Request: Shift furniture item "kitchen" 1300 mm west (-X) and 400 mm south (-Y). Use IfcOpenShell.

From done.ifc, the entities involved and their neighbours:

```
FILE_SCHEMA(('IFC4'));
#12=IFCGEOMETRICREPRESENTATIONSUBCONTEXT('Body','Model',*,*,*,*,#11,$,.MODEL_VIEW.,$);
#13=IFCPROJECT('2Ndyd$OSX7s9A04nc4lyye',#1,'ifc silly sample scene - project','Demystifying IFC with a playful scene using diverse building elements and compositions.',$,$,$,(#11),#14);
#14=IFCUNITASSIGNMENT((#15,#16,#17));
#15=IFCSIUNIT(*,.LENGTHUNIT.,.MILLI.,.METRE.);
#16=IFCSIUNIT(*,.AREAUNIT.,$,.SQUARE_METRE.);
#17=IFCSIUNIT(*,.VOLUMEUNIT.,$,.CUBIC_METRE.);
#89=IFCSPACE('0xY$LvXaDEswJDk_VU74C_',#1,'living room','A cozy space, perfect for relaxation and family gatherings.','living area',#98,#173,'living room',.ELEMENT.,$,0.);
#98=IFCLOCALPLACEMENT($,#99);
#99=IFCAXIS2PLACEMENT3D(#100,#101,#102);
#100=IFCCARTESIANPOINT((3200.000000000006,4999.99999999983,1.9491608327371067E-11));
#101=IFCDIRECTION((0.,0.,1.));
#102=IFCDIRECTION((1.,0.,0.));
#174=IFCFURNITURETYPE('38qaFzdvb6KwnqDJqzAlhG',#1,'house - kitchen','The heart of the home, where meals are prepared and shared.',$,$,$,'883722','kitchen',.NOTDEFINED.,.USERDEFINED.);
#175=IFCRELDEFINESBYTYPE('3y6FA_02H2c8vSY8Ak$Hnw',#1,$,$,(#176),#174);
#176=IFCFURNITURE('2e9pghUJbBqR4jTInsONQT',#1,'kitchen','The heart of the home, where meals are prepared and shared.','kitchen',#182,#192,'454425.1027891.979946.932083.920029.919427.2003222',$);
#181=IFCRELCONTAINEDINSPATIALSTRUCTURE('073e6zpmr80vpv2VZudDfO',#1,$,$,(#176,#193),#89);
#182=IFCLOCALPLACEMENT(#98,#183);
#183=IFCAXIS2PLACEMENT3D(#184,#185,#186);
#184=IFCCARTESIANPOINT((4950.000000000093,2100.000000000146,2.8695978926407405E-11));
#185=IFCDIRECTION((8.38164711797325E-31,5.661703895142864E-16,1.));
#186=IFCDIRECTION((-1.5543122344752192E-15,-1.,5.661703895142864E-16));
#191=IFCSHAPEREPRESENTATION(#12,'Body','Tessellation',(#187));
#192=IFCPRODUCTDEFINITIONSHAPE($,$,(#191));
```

```python
import ifcopenshell
import ifcopenshell.api.geometry
import ifcopenshell.util.placement
import ifcopenshell.util.unit

model = ifcopenshell.open("done.ifc")
unit_scale = ifcopenshell.util.unit.calculate_unit_scale(model)

item = model.by_guid("2e9pghUJbBqR4jTInsONQT")
matrix = ifcopenshell.util.placement.get_local_placement(item.ObjectPlacement)
matrix[0, 3] -= 1.3 / unit_scale
matrix[1, 3] -= 0.4 / unit_scale
ifcopenshell.api.geometry.edit_object_placement(model, product=item, matrix=matrix, is_si=False)

print(ifcopenshell.util.placement.get_local_placement(item.ObjectPlacement).round(3) + 0.0)

model.write("done_v2.ifc")
```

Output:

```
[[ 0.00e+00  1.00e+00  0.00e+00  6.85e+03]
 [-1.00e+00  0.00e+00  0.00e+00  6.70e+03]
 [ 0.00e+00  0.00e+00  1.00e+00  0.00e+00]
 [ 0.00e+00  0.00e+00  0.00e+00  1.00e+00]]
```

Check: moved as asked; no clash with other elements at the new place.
